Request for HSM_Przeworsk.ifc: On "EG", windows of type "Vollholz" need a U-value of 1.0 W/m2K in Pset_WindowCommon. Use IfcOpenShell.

First a look at what the model holds.

```python
import ifcopenshell
import ifcopenshell.util.element

model = ifcopenshell.open("HSM_Przeworsk.ifc")
print(model.schema)
storey = next(s for s in model.by_type("IfcBuildingStorey") if s.Name == "EG")
windows = [e for e in ifcopenshell.util.element.get_decomposition(storey) if e.is_a("IfcWindow")]
seen = {}
for e in windows:
    element_type = ifcopenshell.util.element.get_type(e)
    key = (element_type.Name if element_type != e and element_type else None, ifcopenshell.util.element.get_pset(e, "Pset_WindowCommon", "ThermalTransmittance"))
    seen[key] = seen.get(key, 0) + 1
for (name, value), count in sorted(seen.items(), key=str):
    print(count, "x", name, "|", value)
```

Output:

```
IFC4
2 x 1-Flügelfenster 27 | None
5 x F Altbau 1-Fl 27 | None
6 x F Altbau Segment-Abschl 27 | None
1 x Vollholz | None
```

```python
import ifcopenshell
import ifcopenshell.api.pset
import ifcopenshell.util.element

model = ifcopenshell.open("HSM_Przeworsk.ifc")

storey = next(s for s in model.by_type("IfcBuildingStorey") if s.Name == "EG")
windows = [e for e in ifcopenshell.util.element.get_decomposition(storey) if e.is_a("IfcWindow")]

count = 0
for e in windows:
    element_type = ifcopenshell.util.element.get_type(e)
    if element_type in (None, e) or element_type.Name != "Vollholz":
        continue
    # add_pset returns the element's existing set when there is one.
    pset = ifcopenshell.api.pset.add_pset(model, product=e, name="Pset_WindowCommon")
    ifcopenshell.api.pset.edit_pset(model, pset=pset, properties={"ThermalTransmittance": 1.0})
    count += 1

print(count, "windows updated")

model.write("HSM_Przeworsk_updated.ifc")
```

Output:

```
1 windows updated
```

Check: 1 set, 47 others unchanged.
